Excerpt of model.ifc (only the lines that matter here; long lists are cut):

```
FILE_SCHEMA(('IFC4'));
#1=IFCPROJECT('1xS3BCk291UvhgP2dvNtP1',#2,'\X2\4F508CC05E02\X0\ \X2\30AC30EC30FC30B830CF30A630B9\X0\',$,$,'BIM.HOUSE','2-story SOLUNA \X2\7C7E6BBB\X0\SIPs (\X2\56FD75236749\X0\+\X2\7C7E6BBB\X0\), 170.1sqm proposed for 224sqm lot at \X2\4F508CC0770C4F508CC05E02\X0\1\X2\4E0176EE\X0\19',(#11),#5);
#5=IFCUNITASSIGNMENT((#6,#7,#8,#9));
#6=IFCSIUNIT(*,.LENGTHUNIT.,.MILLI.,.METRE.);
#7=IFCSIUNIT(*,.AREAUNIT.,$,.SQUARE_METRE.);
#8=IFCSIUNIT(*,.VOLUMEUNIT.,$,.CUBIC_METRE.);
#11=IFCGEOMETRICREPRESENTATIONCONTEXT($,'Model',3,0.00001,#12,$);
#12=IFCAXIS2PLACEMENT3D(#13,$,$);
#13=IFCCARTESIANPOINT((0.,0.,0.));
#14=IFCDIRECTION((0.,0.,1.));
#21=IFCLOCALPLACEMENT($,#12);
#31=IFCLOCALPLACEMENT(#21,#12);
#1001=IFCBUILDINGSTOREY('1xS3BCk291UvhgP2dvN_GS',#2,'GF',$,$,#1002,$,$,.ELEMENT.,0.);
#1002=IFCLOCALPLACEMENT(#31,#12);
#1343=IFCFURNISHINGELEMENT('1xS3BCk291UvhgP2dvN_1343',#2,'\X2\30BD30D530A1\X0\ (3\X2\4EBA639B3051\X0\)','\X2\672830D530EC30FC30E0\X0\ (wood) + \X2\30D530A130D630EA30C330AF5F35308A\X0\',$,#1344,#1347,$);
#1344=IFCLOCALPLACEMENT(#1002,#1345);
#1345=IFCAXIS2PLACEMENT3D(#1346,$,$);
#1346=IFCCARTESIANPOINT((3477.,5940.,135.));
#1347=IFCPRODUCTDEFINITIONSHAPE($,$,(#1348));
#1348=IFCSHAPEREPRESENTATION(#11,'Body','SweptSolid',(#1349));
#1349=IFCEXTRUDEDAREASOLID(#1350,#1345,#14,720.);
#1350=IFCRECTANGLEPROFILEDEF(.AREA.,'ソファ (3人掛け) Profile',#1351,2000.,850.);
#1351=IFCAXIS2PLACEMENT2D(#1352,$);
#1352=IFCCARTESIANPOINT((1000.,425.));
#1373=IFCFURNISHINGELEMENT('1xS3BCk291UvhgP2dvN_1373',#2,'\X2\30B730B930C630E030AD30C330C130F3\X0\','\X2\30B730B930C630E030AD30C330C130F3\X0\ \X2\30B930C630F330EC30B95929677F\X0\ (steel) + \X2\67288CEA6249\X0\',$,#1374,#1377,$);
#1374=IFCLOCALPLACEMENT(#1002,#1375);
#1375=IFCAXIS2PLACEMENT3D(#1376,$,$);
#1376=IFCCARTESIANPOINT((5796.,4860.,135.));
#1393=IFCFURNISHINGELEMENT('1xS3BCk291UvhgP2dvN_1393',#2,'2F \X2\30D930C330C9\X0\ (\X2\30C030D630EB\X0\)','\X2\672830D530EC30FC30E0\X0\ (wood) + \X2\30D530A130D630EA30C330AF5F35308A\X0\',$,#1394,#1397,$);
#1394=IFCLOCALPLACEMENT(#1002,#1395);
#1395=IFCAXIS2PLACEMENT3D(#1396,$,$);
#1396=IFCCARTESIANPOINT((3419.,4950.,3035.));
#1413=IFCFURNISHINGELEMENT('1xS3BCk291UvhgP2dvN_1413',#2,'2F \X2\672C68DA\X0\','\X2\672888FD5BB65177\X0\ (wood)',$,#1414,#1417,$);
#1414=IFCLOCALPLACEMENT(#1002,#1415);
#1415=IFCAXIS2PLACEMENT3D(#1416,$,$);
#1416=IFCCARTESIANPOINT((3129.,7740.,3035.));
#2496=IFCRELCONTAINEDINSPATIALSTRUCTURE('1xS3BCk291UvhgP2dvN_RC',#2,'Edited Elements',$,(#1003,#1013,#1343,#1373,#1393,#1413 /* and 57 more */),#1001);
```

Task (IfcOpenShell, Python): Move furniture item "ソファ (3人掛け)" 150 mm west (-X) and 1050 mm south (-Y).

```python
import ifcopenshell
import ifcopenshell.api.geometry
import ifcopenshell.util.placement
import ifcopenshell.util.unit

model = ifcopenshell.open("model.ifc")
unit_scale = ifcopenshell.util.unit.calculate_unit_scale(model)

item = model.by_id(1343)
matrix = ifcopenshell.util.placement.get_local_placement(item.ObjectPlacement)
matrix[0, 3] -= 0.15 / unit_scale
matrix[1, 3] -= 1.05 / unit_scale
ifcopenshell.api.geometry.edit_object_placement(model, product=item, matrix=matrix, is_si=False)

print(ifcopenshell.util.placement.get_local_placement(item.ObjectPlacement).round(3) + 0.0)

model.write("model_v2.ifc")
```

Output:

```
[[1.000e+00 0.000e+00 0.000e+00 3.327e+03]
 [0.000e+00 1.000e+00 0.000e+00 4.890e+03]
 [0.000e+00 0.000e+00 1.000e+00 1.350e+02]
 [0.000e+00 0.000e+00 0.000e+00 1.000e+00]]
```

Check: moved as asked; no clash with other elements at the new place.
